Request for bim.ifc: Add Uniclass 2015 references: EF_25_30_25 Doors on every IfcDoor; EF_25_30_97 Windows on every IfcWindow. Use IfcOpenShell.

First a look at what the model holds.

```python
import ifcopenshell

model = ifcopenshell.open("bim.ifc")
print(model.schema)
print("classifications:", [c.Name for c in model.by_type("IfcClassification")])
for ifc_class in ("IfcDoor", "IfcRoof", "IfcStair", "IfcWall", "IfcWindow"):
    print(ifc_class, len(model.by_type(ifc_class)))
```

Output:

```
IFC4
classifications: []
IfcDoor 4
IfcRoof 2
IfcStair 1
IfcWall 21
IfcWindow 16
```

```python
import ifcopenshell
import ifcopenshell.api.classification

model = ifcopenshell.open("bim.ifc")

system = ifcopenshell.api.classification.add_classification(model, classification="Uniclass 2015")

codes = {
    "IfcDoor": ("EF_25_30_25", "Doors"),
    "IfcWindow": ("EF_25_30_97", "Windows"),
}
for ifc_class, (code, name) in codes.items():
    products = model.by_type(ifc_class)
    ifcopenshell.api.classification.add_reference(
        model, products=products, classification=system, identification=code, name=name
    )
    print(code, len(products))

model.write("bim_updated.ifc")
```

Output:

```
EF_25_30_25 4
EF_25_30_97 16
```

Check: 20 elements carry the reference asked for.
